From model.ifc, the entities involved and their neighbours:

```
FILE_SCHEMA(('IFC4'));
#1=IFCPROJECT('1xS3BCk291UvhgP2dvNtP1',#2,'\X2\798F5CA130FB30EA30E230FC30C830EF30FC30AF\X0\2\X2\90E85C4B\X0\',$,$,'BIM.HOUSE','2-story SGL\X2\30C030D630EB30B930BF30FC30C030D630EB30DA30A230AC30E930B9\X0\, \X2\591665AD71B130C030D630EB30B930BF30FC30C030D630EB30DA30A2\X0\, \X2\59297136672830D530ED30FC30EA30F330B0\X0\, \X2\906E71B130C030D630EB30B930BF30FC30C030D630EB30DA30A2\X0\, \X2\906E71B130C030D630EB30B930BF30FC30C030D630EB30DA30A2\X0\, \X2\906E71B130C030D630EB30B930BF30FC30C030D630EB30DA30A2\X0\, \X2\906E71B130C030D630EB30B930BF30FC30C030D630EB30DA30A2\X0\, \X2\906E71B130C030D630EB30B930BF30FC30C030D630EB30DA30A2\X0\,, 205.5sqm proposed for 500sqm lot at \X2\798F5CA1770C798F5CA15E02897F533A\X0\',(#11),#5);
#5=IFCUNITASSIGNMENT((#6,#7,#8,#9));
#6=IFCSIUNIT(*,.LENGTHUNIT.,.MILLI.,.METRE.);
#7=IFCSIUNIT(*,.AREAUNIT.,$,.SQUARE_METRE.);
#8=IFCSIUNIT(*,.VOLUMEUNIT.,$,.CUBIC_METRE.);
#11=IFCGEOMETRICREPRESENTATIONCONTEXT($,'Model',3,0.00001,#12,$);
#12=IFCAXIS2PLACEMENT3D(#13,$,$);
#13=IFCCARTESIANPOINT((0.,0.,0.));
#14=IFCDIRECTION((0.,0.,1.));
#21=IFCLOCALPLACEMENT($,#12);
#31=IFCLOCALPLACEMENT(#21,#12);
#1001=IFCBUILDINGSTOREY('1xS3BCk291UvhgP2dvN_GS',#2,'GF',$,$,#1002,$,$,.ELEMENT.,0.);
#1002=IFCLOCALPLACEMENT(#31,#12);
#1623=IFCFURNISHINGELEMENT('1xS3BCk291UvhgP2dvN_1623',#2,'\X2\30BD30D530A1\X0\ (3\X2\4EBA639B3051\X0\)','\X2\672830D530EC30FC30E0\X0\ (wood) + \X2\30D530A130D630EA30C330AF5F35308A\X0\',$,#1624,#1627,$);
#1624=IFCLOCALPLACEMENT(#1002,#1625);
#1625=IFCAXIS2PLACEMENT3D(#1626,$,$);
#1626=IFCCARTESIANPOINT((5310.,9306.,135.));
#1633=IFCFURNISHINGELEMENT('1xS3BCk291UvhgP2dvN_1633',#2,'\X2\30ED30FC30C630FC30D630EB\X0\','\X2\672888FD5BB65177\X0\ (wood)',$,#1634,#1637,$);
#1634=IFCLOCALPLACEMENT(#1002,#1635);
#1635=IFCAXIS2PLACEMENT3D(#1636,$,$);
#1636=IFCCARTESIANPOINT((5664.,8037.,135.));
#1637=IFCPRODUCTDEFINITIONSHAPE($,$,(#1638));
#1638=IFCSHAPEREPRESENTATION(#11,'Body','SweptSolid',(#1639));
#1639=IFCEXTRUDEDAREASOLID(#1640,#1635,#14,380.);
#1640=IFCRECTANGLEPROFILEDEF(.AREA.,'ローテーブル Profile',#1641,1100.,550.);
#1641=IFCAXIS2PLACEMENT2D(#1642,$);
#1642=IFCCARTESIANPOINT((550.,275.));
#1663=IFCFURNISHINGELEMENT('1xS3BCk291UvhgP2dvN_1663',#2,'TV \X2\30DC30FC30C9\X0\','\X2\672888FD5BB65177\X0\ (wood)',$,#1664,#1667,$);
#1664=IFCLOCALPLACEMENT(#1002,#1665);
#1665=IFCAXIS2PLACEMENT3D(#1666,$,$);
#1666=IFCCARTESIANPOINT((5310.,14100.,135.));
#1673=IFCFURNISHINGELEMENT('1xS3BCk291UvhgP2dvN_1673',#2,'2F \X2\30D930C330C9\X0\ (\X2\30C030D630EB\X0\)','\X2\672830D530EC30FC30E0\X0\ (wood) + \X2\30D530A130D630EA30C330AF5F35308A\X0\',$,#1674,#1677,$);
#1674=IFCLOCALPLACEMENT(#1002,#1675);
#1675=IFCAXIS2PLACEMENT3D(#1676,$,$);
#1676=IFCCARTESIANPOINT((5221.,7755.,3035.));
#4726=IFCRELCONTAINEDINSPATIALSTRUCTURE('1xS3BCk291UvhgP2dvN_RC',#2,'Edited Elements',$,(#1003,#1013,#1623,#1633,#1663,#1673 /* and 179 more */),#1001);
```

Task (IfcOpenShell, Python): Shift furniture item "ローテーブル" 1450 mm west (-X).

```python
import ifcopenshell
import ifcopenshell.api.geometry
import ifcopenshell.util.placement
import ifcopenshell.util.unit

model = ifcopenshell.open("model.ifc")
unit_scale = ifcopenshell.util.unit.calculate_unit_scale(model)

item = model.by_guid("1xS3BCk291UvhgP2dvN_1633")
matrix = ifcopenshell.util.placement.get_local_placement(item.ObjectPlacement)
matrix[0, 3] -= 1.45 / unit_scale
ifcopenshell.api.geometry.edit_object_placement(model, product=item, matrix=matrix, is_si=False)

print(ifcopenshell.util.placement.get_local_placement(item.ObjectPlacement).round(3) + 0.0)

model.write("model_updated.ifc")
```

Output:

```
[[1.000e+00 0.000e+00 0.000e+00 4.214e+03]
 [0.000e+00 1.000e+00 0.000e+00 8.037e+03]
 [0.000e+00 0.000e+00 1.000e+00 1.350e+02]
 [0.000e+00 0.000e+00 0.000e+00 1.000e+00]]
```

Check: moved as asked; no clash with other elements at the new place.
